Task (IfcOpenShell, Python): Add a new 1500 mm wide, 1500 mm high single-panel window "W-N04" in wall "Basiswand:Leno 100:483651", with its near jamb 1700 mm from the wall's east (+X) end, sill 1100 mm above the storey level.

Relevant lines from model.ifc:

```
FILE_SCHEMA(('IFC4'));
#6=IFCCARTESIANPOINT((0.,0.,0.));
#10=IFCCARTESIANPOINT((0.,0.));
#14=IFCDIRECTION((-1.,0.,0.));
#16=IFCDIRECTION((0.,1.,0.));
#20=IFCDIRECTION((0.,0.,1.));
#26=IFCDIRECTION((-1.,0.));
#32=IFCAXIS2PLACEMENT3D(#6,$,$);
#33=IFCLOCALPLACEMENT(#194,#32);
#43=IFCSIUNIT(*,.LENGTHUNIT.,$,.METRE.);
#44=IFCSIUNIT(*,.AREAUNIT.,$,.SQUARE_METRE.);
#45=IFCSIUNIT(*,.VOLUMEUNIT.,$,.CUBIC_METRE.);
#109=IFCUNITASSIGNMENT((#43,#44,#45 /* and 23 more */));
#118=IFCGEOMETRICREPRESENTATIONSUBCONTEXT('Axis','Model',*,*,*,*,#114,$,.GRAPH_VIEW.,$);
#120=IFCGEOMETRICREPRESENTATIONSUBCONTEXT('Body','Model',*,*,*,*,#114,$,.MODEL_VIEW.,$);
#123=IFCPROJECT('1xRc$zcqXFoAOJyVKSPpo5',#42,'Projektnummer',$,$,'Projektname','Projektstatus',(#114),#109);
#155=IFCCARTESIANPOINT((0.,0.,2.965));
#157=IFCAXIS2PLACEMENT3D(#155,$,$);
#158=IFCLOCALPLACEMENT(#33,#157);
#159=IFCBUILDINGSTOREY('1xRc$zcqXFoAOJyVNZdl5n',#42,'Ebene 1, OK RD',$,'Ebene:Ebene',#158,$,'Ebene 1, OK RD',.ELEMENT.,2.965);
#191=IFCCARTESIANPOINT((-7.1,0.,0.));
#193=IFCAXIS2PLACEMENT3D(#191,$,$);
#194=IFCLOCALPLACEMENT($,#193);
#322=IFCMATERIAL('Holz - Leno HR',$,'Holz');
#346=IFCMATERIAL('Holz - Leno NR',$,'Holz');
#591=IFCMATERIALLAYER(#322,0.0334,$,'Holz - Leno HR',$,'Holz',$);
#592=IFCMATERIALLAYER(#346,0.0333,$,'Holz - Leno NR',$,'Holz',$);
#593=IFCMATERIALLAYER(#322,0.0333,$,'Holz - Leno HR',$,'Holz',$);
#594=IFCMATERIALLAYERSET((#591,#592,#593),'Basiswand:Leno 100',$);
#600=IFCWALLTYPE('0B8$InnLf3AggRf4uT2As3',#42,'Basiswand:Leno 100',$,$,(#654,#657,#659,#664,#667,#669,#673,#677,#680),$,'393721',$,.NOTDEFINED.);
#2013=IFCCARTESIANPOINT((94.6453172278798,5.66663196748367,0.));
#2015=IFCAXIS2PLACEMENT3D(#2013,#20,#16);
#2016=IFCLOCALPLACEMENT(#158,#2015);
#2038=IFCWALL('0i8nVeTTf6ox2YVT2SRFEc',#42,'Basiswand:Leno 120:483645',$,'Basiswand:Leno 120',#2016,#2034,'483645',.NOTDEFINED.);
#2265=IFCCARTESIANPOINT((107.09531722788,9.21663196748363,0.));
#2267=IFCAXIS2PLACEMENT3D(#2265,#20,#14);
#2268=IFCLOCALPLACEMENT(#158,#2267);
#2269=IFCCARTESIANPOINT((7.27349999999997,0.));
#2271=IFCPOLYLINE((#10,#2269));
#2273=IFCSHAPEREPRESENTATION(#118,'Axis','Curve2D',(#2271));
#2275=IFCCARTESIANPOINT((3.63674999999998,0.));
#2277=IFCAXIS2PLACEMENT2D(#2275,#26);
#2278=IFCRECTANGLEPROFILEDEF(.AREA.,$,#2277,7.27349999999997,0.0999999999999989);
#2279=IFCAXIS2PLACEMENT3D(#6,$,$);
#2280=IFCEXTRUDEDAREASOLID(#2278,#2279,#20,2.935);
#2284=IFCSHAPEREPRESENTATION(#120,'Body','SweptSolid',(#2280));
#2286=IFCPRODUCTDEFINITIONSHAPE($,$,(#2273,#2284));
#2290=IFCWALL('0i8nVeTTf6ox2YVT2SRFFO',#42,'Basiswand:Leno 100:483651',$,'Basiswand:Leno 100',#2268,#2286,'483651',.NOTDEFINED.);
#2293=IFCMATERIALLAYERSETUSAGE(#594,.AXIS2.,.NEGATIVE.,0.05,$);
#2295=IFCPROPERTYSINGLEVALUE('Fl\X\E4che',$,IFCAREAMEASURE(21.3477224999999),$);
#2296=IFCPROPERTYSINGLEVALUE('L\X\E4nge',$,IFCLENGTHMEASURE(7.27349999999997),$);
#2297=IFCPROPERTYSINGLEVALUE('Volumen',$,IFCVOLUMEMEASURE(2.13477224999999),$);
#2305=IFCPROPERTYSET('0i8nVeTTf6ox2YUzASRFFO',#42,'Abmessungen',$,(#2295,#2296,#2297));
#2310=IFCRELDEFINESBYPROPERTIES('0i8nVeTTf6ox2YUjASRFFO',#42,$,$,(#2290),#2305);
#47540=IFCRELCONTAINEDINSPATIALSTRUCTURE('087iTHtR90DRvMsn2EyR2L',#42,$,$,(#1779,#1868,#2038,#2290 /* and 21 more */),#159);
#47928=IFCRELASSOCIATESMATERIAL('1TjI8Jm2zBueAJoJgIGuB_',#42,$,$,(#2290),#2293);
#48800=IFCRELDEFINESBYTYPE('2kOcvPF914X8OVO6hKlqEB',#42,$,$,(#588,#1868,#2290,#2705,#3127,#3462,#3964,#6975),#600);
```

```python
import numpy as np
import ifcopenshell
import ifcopenshell.api.feature
import ifcopenshell.api.geometry
import ifcopenshell.api.pset
import ifcopenshell.api.root
import ifcopenshell.api.spatial
import ifcopenshell.geom
import ifcopenshell.util.element
import ifcopenshell.util.placement
import ifcopenshell.util.representation
import ifcopenshell.util.shape
import ifcopenshell.util.unit

model = ifcopenshell.open("model.ifc")
unit_scale = ifcopenshell.util.unit.calculate_unit_scale(model)
area_scale = ifcopenshell.util.unit.calculate_unit_scale(model, "AREAUNIT")
volume_scale = ifcopenshell.util.unit.calculate_unit_scale(model, "VOLUMEUNIT")
settings = ifcopenshell.geom.settings()


def volume(element):
    """Net volume in cubic metres, openings subtracted."""
    shape = ifcopenshell.geom.create_shape(settings, element)
    return ifcopenshell.util.shape.get_volume(shape.geometry)


wall = model.by_id(2290)
storey = ifcopenshell.util.element.get_container(wall, ifc_class="IfcBuildingStorey")
context = ifcopenshell.util.representation.get_context(model, "Model", "Body", "MODEL_VIEW")
before = volume(wall)

width, height, from_end, sill = 1.5, 1.5, 1.7, 1.1  # metres

# The wall runs along its own X axis, and the end named is its -X end.
wall_shape = ifcopenshell.geom.create_shape(settings, wall)
x, y, z = ifcopenshell.util.shape.get_vertices(wall_shape.geometry).T
start = x.min() + from_end
face, thickness = float(y.min()), float(y.max() - y.min())
wall_matrix = ifcopenshell.util.placement.get_local_placement(wall.ObjectPlacement)
level = ifcopenshell.util.placement.get_local_placement(storey.ObjectPlacement)[2, 3]


def in_wall(x, y):
    """Placement at x, y metres in the wall's axes, at sill height."""
    matrix = wall_matrix.copy()
    matrix[:, 3] = wall_matrix @ np.array([x / unit_scale, y / unit_scale, 0.0, 1.0])
    matrix[2, 3] = level + sill / unit_scale
    return matrix


# Opening: a box that overshoots both wall faces by 50 mm.
opening = ifcopenshell.api.root.create_entity(model, ifc_class="IfcOpeningElement", predefined_type="OPENING")
box = ifcopenshell.api.geometry.add_wall_representation(
    model, context=context, length=width, height=height, thickness=thickness + 0.1
)
ifcopenshell.api.geometry.assign_representation(model, product=opening, representation=box)
ifcopenshell.api.geometry.edit_object_placement(model, product=opening, matrix=in_wall(start, face - 0.05), is_si=False)
ifcopenshell.api.feature.add_feature(model, feature=opening, element=wall)

window = ifcopenshell.api.root.create_entity(model, ifc_class="IfcWindow", name="W-N04", predefined_type="WINDOW")
window.OverallWidth, window.OverallHeight = width / unit_scale, height / unit_scale
window.PartitioningType = "SINGLE_PANEL"
body = ifcopenshell.api.geometry.add_window_representation(
    model,
    context=context,
    overall_width=window.OverallWidth,
    overall_height=window.OverallHeight,
    partition_type="SINGLE_PANEL",
)
ifcopenshell.api.geometry.assign_representation(model, product=window, representation=body)
ifcopenshell.api.spatial.assign_container(model, products=[window], relating_structure=storey)
ifcopenshell.api.feature.add_filling(model, opening=opening, element=window)

# Centre the window in the wall's thickness.
ifcopenshell.api.geometry.edit_object_placement(model, product=window, matrix=in_wall(start, face), is_si=False)
window_shape = ifcopenshell.geom.create_shape(settings, window)
depth = ifcopenshell.util.shape.get_vertices(window_shape.geometry)[:, 1]
offset = face + thickness / 2 - (depth.min() + depth.max()) / 2
ifcopenshell.api.geometry.edit_object_placement(model, product=window, matrix=in_wall(start, offset), is_si=False)

after = volume(wall)

# Update the wall's stored quantities.
pset = model.by_id(ifcopenshell.util.element.get_pset(wall, "Abmessungen", should_inherit=False)["id"])
ifcopenshell.api.pset.edit_pset(model, pset=pset, properties={
    "Fläche": model.create_entity("IfcAreaMeasure", after / thickness / area_scale),
    "Volumen": model.create_entity("IfcVolumeMeasure", after / volume_scale),
})

print(f"wall volume {before:.3f} -> {after:.3f} m3")

model.write("model_rev.ifc")
```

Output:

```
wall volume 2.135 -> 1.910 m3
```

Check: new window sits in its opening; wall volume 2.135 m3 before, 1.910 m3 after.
